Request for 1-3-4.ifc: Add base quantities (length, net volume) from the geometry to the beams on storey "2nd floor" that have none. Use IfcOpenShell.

First a look at what the model holds.

```python
import ifcopenshell
import ifcopenshell.util.element
import ifcopenshell.util.unit

model = ifcopenshell.open("1-3-4.ifc")
print(model.schema)
for unit_type in ("LENGTHUNIT", "AREAUNIT", "VOLUMEUNIT"):
    print(unit_type, ifcopenshell.util.unit.calculate_unit_scale(model, unit_type))
storey = next(s for s in model.by_type("IfcBuildingStorey") if s.Name == "2nd floor")
beams = [e for e in ifcopenshell.util.element.get_decomposition(storey) if e.is_a("IfcBeam")]
for e in sorted(beams, key=lambda e: e.id()):
    print(e.id(), e.is_a(), e.Name, list(ifcopenshell.util.element.get_psets(e, qtos_only=True)), sep=" | ")
```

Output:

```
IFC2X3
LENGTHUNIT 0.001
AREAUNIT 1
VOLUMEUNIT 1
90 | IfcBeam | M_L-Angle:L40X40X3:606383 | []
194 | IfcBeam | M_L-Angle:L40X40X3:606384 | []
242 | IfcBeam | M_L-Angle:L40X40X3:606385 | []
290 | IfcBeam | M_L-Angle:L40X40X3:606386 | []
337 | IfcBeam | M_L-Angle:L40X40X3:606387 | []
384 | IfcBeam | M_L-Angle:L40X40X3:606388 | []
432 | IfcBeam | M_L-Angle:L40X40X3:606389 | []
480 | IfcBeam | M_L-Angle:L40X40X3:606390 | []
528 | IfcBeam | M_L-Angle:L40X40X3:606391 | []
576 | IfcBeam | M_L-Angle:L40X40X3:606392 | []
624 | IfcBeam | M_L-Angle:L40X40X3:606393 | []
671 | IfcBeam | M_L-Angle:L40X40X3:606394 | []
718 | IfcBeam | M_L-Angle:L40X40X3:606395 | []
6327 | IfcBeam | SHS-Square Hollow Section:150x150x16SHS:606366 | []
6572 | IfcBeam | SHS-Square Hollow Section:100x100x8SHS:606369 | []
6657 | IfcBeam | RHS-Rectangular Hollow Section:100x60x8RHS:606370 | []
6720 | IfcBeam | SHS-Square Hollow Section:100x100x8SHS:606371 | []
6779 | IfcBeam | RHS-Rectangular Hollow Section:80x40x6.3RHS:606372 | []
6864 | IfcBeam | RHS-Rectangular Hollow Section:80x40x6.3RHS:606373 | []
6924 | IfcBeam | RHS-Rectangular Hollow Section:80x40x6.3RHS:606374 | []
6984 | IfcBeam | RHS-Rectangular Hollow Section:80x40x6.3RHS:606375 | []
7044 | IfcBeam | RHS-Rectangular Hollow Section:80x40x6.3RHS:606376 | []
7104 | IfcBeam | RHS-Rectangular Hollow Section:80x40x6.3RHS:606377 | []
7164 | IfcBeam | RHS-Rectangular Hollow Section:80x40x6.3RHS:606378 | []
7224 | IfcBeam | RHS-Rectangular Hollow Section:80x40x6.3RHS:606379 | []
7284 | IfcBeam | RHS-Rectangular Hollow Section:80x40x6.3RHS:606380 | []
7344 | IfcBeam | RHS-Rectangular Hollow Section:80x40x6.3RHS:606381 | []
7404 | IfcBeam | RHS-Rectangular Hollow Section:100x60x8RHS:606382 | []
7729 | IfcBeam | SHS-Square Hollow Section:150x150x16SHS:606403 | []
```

```python
import ifcopenshell
import ifcopenshell.api.pset
import ifcopenshell.geom
import ifcopenshell.util.element
import ifcopenshell.util.shape
import ifcopenshell.util.unit

model = ifcopenshell.open("1-3-4.ifc")
unit_scale = ifcopenshell.util.unit.calculate_unit_scale(model)
volume_scale = ifcopenshell.util.unit.calculate_unit_scale(model, "VOLUMEUNIT")
settings = ifcopenshell.geom.settings()

storey = next(s for s in model.by_type("IfcBuildingStorey") if s.Name == "2nd floor")
beams = [e for e in ifcopenshell.util.element.get_decomposition(storey) if e.is_a("IfcBeam")]

for e in sorted(beams, key=lambda e: e.id()):
    if ifcopenshell.util.element.get_psets(e, qtos_only=True, should_inherit=False):
        continue
    # Geometry comes back in metres, in the element's own axes.
    shape = ifcopenshell.geom.create_shape(settings, e)
    values = {
        "Length": ifcopenshell.util.shape.get_max_xyz(shape.geometry) / unit_scale,
        "NetVolume": ifcopenshell.util.shape.get_volume(shape.geometry) / volume_scale,
    }
    qto = ifcopenshell.api.pset.add_qto(model, product=e, name="BaseQuantities")
    ifcopenshell.api.pset.edit_qto(model, qto=qto, properties=values)
    print(e.id(), {k: round(v, 3) for k, v in values.items()})

model.write("1-3-4_edited.ifc")
```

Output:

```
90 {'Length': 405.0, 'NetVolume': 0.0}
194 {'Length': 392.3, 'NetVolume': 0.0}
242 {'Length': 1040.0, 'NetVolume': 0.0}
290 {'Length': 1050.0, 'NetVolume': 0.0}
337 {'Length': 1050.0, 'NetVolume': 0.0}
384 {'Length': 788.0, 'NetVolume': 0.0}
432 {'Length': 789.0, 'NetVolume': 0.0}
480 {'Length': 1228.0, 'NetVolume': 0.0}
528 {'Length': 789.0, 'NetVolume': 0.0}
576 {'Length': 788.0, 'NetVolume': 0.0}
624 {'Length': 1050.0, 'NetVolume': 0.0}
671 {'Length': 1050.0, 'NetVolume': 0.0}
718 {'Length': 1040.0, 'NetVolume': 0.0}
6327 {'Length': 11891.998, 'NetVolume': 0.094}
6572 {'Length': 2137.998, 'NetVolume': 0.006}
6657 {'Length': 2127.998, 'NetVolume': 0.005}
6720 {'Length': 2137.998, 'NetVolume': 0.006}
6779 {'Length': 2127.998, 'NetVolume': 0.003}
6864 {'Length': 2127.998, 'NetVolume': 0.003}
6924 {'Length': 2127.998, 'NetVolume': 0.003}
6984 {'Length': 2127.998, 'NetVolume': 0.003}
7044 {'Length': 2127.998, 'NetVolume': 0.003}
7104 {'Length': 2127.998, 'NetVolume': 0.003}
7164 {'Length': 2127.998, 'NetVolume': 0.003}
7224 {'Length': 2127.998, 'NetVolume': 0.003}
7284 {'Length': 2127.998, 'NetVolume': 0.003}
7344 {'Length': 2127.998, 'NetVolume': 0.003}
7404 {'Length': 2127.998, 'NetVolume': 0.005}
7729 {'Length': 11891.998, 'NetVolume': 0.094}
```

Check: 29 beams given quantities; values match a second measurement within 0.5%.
